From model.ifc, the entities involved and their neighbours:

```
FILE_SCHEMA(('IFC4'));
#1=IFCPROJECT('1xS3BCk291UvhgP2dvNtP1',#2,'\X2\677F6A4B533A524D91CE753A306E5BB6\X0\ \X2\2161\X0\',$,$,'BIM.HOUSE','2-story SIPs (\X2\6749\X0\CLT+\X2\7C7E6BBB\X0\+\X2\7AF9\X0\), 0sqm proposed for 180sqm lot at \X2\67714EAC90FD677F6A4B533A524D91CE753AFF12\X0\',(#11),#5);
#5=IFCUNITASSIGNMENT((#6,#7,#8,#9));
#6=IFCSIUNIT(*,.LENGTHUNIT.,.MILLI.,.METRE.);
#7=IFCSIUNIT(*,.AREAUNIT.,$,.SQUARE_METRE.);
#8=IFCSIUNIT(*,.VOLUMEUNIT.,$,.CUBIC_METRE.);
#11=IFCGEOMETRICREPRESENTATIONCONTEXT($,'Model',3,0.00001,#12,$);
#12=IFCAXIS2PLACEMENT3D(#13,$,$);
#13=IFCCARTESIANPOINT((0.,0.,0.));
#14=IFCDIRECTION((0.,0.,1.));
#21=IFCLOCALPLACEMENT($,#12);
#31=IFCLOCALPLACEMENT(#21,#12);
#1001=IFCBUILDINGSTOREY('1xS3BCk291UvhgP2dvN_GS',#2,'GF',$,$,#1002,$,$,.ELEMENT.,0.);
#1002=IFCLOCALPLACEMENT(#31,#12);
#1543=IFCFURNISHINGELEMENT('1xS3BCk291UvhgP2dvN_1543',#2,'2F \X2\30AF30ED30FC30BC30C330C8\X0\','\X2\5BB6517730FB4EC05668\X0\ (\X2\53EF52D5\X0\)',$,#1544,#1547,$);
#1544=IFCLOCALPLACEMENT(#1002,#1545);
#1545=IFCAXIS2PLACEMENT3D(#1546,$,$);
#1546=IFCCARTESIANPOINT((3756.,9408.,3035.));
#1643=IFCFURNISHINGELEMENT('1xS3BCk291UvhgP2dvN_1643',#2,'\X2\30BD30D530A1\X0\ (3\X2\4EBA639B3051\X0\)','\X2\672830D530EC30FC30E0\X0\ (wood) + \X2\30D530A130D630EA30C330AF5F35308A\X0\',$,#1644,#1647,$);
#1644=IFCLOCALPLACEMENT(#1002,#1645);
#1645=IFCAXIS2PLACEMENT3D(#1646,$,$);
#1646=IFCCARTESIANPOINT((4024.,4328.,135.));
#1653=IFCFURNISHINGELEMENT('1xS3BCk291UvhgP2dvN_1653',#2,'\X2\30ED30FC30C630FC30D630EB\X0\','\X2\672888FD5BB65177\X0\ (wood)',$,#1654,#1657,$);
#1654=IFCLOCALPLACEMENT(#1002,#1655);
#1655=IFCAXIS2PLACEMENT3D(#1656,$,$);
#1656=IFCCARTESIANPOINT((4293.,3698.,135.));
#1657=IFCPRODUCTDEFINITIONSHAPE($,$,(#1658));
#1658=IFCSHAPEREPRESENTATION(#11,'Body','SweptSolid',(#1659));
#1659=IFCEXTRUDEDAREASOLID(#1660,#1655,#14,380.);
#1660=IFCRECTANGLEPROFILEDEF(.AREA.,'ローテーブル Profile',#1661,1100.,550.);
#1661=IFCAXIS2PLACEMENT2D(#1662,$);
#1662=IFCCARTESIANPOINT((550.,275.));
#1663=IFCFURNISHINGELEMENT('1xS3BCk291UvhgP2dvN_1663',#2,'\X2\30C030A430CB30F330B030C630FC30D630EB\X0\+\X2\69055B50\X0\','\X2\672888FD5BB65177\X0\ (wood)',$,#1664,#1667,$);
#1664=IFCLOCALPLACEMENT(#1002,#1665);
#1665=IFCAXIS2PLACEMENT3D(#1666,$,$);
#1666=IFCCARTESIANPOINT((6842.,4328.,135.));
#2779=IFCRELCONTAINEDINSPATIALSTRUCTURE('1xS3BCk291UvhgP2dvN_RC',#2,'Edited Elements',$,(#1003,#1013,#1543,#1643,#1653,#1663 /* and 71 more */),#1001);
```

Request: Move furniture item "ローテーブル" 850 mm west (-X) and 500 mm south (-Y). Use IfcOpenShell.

```python
import ifcopenshell
import ifcopenshell.api.geometry
import ifcopenshell.util.placement
import ifcopenshell.util.unit

model = ifcopenshell.open("model.ifc")
unit_scale = ifcopenshell.util.unit.calculate_unit_scale(model)

item = model.by_id(1653)
matrix = ifcopenshell.util.placement.get_local_placement(item.ObjectPlacement)
matrix[0, 3] -= 0.85 / unit_scale
matrix[1, 3] -= 0.5 / unit_scale
ifcopenshell.api.geometry.edit_object_placement(model, product=item, matrix=matrix, is_si=False)

print(ifcopenshell.util.placement.get_local_placement(item.ObjectPlacement).round(3) + 0.0)

model.write("model_updated.ifc")
```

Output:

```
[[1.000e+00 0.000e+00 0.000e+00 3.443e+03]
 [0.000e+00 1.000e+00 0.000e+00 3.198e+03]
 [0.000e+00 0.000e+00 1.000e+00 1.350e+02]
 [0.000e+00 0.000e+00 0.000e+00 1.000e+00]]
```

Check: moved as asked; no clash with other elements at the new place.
